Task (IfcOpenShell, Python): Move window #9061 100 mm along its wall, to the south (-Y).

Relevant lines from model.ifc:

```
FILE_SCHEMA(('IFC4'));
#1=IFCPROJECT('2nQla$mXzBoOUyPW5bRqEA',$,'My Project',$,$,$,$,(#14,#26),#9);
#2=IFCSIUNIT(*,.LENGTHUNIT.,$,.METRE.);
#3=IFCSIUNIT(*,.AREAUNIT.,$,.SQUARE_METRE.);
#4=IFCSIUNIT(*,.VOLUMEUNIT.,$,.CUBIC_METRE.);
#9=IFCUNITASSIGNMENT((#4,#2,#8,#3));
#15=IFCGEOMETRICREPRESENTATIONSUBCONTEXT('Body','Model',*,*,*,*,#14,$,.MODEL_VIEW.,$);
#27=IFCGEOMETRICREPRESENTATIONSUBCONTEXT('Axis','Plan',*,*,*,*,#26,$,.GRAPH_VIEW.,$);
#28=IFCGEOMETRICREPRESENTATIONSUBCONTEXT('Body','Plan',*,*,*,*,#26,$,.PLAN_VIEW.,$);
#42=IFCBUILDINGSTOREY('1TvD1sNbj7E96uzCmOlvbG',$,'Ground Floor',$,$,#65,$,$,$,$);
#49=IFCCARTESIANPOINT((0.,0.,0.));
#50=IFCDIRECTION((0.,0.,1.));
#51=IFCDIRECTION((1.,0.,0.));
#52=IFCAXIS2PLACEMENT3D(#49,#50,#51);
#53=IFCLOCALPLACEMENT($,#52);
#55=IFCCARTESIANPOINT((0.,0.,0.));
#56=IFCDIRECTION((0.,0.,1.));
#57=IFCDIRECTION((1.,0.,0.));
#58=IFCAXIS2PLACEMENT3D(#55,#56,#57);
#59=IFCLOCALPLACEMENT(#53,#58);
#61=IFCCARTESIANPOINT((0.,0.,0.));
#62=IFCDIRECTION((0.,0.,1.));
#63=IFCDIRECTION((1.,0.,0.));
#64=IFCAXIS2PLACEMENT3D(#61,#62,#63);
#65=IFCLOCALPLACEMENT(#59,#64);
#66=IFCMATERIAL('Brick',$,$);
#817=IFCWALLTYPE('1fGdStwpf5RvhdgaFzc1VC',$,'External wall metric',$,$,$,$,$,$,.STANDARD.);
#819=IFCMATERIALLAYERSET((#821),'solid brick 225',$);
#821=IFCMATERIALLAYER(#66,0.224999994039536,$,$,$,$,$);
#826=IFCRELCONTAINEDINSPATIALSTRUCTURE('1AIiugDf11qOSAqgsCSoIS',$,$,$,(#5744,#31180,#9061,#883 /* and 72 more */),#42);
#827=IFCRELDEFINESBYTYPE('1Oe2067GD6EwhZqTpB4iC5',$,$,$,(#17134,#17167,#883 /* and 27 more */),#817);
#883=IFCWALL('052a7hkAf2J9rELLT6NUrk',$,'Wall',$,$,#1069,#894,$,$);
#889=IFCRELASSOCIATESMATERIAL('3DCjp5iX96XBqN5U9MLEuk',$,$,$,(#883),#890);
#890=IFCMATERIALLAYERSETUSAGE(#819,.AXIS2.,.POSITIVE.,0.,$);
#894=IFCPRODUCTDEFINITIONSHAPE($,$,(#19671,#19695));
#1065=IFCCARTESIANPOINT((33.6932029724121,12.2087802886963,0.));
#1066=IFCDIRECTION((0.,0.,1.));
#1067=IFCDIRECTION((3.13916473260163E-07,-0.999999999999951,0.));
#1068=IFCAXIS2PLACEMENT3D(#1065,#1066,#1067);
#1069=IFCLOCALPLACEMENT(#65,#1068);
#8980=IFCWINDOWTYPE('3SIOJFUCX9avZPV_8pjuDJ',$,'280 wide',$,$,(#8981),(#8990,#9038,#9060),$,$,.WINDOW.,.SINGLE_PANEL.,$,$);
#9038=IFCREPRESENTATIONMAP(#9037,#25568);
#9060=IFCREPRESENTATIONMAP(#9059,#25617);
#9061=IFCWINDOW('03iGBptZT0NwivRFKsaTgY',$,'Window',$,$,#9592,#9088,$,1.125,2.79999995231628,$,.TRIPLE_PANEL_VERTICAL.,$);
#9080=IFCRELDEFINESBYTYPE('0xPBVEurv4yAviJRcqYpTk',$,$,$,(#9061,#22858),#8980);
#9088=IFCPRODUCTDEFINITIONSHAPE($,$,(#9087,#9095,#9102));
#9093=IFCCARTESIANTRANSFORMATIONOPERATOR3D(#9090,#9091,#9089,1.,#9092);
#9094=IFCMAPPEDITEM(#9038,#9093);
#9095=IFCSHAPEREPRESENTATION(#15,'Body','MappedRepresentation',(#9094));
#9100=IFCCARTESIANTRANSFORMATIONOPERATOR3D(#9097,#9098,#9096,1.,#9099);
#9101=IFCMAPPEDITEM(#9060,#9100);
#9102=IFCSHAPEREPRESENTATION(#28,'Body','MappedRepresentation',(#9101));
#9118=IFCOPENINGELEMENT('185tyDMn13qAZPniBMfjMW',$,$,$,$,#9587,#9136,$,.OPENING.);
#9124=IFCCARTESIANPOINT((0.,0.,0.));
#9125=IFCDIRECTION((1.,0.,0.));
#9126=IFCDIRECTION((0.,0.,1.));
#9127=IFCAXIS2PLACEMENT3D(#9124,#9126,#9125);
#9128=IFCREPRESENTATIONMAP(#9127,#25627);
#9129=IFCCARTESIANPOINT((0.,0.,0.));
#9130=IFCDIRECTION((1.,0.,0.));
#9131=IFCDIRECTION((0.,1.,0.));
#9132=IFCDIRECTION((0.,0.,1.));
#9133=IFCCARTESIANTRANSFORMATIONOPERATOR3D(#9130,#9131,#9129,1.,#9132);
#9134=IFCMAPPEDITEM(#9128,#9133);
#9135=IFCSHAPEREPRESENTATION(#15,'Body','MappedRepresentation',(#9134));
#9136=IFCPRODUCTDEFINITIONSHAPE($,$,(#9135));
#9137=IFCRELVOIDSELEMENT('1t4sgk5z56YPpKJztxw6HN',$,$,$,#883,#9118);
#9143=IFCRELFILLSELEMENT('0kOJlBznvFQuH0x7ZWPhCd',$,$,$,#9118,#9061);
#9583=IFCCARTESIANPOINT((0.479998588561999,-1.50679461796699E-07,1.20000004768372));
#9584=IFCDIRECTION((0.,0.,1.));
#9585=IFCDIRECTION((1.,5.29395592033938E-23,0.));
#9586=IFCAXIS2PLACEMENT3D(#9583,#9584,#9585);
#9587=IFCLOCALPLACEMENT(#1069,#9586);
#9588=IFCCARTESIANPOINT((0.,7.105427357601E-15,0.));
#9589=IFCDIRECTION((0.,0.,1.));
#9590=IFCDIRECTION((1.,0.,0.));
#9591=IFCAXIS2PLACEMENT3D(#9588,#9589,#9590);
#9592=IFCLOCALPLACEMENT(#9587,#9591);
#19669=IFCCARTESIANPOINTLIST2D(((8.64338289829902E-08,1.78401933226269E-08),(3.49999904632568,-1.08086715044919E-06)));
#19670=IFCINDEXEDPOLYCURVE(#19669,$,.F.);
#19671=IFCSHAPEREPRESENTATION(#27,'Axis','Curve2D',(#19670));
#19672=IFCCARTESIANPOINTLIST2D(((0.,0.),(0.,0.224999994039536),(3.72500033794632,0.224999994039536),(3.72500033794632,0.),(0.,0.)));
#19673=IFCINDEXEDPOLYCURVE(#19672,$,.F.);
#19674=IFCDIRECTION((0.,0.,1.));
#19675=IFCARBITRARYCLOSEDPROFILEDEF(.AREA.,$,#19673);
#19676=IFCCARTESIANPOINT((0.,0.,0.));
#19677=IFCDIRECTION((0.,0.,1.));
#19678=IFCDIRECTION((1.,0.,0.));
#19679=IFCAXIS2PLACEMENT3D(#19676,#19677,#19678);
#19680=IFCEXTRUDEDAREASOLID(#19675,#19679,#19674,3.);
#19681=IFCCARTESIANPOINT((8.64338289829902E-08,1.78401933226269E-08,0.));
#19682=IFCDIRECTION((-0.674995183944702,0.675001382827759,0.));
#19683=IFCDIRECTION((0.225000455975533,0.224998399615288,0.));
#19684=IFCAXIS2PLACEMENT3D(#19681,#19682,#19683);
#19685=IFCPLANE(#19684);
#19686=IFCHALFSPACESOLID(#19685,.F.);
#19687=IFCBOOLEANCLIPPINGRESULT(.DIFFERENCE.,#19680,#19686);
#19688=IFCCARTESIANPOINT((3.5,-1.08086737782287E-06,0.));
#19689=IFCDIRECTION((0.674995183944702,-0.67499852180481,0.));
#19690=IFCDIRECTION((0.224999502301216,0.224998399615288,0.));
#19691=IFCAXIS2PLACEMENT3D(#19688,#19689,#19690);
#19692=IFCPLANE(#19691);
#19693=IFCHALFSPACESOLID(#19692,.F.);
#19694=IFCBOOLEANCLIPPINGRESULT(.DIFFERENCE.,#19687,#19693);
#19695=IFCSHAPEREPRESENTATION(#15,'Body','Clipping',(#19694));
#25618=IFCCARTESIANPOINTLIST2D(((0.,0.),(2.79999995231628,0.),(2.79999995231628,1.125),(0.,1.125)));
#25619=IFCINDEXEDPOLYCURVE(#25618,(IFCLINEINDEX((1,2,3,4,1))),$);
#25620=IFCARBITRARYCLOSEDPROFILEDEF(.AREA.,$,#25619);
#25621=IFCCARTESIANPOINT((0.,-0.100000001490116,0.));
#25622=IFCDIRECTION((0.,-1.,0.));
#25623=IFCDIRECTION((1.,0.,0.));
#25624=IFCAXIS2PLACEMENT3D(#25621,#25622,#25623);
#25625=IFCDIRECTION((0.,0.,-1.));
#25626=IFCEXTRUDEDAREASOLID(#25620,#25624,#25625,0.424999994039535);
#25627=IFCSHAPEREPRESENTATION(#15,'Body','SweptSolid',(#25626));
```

```python
import ifcopenshell
import ifcopenshell.api.geometry
import ifcopenshell.util.placement

model = ifcopenshell.open("model.ifc")

window = model.by_guid("03iGBptZT0NwivRFKsaTgY")
opening = window.FillsVoids[0].RelatingOpeningElement
wall = opening.VoidsElements[0].RelatingBuildingElement

wall_matrix = ifcopenshell.util.placement.get_local_placement(wall.ObjectPlacement)
shift = wall_matrix[:3, 0] * 0.1
before = ifcopenshell.util.placement.get_local_placement(window.ObjectPlacement)[:3, 3].copy()

# The window is placed relative to its opening, so it follows when the opening moves.
matrix = ifcopenshell.util.placement.get_local_placement(opening.ObjectPlacement)
matrix[:3, 3] += shift
ifcopenshell.api.geometry.edit_object_placement(
    model, product=opening, matrix=matrix, is_si=False, should_transform_children=True
)

after = ifcopenshell.util.placement.get_local_placement(window.ObjectPlacement)[:3, 3]
print("window moved by", (after - before).round(3) + 0.0)

model.write("model_rev.ifc")
```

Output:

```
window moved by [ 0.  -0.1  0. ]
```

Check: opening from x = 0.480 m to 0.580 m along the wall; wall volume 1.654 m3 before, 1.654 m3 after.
